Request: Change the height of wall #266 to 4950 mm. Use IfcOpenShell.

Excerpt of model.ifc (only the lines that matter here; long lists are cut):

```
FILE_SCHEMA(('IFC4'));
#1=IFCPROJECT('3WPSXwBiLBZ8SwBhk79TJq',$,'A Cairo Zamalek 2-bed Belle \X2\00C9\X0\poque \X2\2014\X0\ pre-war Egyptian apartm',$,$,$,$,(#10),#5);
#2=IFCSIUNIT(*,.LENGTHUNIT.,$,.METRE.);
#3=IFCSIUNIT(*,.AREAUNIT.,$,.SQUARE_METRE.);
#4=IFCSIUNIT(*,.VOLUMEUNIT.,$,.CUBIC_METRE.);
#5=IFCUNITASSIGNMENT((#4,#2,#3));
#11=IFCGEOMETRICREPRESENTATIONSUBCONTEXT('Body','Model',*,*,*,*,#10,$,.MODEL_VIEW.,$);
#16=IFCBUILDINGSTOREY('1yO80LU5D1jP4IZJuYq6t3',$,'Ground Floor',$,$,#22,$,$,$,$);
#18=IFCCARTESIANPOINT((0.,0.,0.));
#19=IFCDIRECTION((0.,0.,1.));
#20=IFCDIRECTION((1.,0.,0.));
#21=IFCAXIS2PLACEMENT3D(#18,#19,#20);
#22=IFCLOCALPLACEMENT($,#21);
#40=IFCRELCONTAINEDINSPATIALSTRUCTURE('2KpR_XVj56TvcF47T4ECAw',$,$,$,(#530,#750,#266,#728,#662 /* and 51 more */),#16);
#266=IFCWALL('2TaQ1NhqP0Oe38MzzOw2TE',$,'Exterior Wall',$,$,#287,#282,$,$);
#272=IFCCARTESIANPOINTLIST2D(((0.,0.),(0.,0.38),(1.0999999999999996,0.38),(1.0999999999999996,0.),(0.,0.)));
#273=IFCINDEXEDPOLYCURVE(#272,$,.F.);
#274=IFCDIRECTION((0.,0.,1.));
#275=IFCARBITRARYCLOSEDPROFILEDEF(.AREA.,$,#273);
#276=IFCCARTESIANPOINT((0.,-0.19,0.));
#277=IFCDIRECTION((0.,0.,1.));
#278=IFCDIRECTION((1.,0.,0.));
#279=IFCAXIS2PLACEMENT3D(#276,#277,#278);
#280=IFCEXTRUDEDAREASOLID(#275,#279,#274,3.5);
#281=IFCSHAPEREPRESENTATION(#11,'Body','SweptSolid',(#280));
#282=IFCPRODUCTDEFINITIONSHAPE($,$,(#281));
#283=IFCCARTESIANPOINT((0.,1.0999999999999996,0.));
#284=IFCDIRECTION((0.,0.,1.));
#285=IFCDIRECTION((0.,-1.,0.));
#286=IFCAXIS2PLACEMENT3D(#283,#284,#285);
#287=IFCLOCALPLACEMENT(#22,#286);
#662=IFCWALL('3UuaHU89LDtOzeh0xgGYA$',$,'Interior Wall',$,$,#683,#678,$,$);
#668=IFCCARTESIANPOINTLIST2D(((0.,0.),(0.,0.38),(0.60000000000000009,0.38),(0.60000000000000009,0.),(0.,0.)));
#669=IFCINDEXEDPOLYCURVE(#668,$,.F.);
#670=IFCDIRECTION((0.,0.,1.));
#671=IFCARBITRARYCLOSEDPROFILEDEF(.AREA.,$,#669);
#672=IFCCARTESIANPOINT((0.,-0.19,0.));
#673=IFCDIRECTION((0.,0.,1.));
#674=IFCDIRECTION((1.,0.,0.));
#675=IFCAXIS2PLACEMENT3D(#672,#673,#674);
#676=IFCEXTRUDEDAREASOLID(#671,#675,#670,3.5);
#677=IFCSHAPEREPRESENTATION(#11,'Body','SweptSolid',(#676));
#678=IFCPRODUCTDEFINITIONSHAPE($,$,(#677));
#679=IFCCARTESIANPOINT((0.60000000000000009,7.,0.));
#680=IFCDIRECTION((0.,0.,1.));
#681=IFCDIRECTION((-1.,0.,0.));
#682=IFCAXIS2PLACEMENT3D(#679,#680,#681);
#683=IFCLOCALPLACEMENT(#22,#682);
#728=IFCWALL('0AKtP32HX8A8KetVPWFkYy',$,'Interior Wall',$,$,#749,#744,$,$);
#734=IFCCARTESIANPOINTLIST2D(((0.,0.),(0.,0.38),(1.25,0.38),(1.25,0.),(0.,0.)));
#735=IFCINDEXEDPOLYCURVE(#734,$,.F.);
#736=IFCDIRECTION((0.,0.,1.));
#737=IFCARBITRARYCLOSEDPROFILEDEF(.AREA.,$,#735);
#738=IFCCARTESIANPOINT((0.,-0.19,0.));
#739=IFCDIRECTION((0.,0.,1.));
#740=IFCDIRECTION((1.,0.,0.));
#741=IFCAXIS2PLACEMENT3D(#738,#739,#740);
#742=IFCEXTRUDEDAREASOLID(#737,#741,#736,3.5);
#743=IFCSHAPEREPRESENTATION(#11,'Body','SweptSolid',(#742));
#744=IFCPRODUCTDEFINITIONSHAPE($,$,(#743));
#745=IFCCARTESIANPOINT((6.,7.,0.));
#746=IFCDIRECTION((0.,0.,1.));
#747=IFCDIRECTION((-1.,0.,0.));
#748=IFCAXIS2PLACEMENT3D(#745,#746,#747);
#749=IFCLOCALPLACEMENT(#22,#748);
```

```python
import ifcopenshell
import ifcopenshell.geom
import ifcopenshell.util.representation
import ifcopenshell.util.shape

model = ifcopenshell.open("model.ifc")
settings = ifcopenshell.geom.settings()


def volume(element):
    """Net volume in cubic metres, openings subtracted."""
    shape = ifcopenshell.geom.create_shape(settings, element)
    return ifcopenshell.util.shape.get_volume(shape.geometry)


wall = model.by_guid("2TaQ1NhqP0Oe38MzzOw2TE")
before = volume(wall)

body = ifcopenshell.util.representation.get_representation(wall, "Model", "Body")
solid = body.Items[0]
old_height = solid.Depth
solid.Depth = 4.95
after = volume(wall)

print(f"height {old_height:g} -> {solid.Depth:g}, volume {before:.3f} -> {after:.3f} m3")

model.write("model_v2.ifc")
```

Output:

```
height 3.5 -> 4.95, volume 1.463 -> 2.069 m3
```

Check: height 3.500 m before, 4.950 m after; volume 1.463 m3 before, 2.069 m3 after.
